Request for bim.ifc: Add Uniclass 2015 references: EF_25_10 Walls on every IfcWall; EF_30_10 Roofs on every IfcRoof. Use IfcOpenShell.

First a look at what the model holds.

```python
import ifcopenshell

model = ifcopenshell.open("bim.ifc")
print(model.schema)
print("classifications:", [c.Name for c in model.by_type("IfcClassification")])
for ifc_class in ("IfcDoor", "IfcRoof", "IfcStair", "IfcWall", "IfcWindow"):
    print(ifc_class, len(model.by_type(ifc_class)))
```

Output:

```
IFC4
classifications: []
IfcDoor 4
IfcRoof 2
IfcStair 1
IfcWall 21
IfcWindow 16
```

```python
import ifcopenshell
import ifcopenshell.api.classification

model = ifcopenshell.open("bim.ifc")

system = ifcopenshell.api.classification.add_classification(model, classification="Uniclass 2015")

codes = {
    "IfcWall": ("EF_25_10", "Walls"),
    "IfcRoof": ("EF_30_10", "Roofs"),
}
for ifc_class, (code, name) in codes.items():
    products = model.by_type(ifc_class)
    ifcopenshell.api.classification.add_reference(
        model, products=products, classification=system, identification=code, name=name
    )
    print(code, len(products))

model.write("bim_edited.ifc")
```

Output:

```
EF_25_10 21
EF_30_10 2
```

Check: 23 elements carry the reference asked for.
